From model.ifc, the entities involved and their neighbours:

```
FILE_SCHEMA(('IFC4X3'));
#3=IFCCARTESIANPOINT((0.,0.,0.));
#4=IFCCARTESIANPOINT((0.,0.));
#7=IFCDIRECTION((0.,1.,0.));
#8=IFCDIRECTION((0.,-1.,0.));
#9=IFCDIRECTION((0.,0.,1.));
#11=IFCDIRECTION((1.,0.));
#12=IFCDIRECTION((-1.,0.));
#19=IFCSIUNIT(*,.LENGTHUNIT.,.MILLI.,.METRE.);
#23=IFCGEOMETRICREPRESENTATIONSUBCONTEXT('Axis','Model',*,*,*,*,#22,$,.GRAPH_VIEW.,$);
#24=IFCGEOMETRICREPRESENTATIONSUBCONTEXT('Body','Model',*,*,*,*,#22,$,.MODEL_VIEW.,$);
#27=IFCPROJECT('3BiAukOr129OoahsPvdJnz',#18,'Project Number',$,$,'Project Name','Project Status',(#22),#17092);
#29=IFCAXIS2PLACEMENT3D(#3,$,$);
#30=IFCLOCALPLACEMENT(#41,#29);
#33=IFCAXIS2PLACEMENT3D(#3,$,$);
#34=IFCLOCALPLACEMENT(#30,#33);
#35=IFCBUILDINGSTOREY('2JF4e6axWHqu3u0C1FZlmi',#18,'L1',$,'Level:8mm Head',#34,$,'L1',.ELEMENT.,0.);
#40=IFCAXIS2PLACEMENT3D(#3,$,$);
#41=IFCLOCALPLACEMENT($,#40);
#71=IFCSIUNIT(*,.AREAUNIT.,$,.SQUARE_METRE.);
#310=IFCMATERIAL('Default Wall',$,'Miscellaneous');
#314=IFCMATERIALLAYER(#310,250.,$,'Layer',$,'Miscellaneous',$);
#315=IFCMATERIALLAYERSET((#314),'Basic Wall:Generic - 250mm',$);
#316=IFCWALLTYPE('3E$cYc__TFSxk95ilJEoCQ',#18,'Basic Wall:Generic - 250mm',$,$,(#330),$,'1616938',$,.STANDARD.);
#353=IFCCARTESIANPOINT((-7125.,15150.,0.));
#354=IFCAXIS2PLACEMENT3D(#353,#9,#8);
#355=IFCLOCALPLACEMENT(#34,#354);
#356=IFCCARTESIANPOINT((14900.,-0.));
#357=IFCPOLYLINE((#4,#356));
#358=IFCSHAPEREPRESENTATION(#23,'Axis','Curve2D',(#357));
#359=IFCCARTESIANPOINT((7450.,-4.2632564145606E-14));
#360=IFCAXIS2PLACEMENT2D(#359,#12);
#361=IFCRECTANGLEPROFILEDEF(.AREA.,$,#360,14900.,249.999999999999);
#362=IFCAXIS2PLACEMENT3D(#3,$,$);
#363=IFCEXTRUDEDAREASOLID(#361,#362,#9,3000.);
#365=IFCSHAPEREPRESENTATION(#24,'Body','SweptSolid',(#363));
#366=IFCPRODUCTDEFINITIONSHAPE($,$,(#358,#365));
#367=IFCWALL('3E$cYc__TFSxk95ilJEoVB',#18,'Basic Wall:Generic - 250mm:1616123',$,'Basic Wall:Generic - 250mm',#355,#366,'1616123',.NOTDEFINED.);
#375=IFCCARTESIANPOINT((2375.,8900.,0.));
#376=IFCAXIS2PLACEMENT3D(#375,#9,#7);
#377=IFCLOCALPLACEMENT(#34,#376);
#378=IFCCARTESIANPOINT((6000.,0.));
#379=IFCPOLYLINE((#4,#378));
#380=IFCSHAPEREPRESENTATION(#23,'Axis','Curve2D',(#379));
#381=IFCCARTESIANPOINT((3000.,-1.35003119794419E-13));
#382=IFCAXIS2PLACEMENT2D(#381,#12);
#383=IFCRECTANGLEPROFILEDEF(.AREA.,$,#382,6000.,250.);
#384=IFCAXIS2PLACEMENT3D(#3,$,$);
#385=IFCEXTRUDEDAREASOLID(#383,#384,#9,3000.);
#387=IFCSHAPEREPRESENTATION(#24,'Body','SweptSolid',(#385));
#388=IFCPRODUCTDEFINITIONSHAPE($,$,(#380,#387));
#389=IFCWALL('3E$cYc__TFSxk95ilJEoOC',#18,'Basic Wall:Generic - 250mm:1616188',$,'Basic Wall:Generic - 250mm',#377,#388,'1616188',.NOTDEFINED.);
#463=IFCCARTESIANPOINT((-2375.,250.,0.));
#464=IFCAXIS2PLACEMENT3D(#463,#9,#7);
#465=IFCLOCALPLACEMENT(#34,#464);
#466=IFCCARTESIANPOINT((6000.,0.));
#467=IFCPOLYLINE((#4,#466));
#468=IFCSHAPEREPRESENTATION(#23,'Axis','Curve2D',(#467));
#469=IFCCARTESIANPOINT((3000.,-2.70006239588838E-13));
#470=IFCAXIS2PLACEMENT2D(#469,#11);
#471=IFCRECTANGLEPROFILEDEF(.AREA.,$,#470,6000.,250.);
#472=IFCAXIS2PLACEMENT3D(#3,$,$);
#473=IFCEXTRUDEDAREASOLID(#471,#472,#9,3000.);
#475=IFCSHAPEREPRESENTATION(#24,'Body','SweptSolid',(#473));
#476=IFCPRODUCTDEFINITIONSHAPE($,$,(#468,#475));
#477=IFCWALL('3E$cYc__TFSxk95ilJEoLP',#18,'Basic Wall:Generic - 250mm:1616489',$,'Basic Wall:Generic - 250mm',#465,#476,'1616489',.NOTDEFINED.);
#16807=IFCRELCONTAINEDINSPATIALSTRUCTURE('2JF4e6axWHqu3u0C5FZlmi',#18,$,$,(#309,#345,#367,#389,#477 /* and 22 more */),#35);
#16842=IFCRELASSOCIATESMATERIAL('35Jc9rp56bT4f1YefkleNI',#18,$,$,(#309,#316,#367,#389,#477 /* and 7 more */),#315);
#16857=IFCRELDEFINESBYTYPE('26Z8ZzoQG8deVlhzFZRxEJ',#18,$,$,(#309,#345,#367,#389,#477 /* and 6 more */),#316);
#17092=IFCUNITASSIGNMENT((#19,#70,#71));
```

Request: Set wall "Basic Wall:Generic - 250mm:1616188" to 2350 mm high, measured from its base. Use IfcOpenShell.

```python
import ifcopenshell
import ifcopenshell.geom
import ifcopenshell.util.representation
import ifcopenshell.util.shape

model = ifcopenshell.open("model.ifc")
settings = ifcopenshell.geom.settings()


def volume(element):
    """Net volume in cubic metres, openings subtracted."""
    shape = ifcopenshell.geom.create_shape(settings, element)
    return ifcopenshell.util.shape.get_volume(shape.geometry)


wall = model.by_guid("3E$cYc__TFSxk95ilJEoOC")
before = volume(wall)

body = ifcopenshell.util.representation.get_representation(wall, "Model", "Body")
solid = body.Items[0]
old_height = solid.Depth
solid.Depth = 2350.0
after = volume(wall)

print(f"height {old_height:g} -> {solid.Depth:g}, volume {before:.3f} -> {after:.3f} m3")

model.write("model_edited.ifc")
```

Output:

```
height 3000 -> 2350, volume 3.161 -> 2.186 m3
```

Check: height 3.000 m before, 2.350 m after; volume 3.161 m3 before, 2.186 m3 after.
